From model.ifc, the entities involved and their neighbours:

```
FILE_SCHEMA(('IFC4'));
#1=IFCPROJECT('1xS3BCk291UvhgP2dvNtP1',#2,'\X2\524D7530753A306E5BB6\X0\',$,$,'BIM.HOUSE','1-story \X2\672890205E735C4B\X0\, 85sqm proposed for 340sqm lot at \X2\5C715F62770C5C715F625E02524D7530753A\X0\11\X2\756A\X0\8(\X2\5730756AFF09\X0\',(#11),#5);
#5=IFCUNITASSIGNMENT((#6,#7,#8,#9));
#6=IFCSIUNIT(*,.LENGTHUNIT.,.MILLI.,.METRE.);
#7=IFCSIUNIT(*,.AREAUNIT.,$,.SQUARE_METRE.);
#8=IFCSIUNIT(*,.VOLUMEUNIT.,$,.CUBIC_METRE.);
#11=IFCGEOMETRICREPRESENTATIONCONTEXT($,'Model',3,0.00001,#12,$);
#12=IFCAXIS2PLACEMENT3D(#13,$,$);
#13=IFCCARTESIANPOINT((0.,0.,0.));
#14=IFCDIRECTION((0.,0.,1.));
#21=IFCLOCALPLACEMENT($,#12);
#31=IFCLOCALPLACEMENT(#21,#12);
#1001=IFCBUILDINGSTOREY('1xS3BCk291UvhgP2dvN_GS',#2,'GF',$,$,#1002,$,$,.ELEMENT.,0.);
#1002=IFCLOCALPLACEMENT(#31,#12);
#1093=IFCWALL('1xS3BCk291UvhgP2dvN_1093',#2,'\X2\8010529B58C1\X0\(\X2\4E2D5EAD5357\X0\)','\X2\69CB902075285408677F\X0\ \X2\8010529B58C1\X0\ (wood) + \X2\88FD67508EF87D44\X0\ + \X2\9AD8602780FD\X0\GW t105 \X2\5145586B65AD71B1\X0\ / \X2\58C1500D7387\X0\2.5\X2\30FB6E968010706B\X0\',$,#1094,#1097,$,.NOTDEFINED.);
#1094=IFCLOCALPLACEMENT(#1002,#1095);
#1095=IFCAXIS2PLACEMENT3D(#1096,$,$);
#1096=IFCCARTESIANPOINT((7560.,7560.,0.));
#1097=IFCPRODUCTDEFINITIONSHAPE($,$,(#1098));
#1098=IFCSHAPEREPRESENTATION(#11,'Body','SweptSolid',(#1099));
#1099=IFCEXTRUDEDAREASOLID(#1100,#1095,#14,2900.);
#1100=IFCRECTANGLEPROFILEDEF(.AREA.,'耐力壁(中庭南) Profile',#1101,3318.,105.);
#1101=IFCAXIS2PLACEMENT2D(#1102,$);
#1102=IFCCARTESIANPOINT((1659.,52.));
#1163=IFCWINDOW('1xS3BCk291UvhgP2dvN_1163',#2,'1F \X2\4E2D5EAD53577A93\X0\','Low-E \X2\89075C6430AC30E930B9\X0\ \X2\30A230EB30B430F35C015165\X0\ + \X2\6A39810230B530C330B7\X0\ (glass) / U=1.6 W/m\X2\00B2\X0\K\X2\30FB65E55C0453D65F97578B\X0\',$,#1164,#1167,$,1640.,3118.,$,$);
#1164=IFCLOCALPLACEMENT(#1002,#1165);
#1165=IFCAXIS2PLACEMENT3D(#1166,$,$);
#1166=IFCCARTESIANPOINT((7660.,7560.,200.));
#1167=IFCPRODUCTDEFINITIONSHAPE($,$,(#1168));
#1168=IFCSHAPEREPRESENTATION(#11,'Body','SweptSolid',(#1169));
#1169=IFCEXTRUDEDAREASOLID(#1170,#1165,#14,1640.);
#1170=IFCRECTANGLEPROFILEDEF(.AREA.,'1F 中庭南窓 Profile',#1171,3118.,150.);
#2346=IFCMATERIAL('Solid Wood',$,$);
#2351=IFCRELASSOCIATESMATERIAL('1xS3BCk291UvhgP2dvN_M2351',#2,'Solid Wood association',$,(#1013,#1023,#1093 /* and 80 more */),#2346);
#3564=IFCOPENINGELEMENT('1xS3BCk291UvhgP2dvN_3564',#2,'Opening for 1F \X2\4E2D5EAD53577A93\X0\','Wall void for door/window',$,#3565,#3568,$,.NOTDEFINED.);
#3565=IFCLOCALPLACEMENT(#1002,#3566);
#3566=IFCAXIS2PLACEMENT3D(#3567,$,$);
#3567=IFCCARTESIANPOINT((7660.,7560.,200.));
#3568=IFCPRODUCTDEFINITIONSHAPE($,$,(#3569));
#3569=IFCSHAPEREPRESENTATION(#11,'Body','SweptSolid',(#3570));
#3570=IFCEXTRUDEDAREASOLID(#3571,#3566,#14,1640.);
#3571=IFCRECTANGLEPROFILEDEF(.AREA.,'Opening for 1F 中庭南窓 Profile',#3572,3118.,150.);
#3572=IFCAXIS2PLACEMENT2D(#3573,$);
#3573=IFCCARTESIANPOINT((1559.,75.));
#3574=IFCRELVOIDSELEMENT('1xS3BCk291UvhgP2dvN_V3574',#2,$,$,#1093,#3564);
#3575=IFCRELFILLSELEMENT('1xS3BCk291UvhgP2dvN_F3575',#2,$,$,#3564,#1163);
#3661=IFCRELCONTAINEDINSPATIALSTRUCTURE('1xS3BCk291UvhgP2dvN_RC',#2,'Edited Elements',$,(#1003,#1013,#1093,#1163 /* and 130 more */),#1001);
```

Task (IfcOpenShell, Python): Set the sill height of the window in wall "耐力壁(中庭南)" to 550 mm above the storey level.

```python
import numpy as np
import ifcopenshell
import ifcopenshell.api.geometry
import ifcopenshell.geom
import ifcopenshell.util.element
import ifcopenshell.util.placement
import ifcopenshell.util.shape
import ifcopenshell.util.unit

model = ifcopenshell.open("model.ifc")
unit_scale = ifcopenshell.util.unit.calculate_unit_scale(model)

window = model.by_guid("1xS3BCk291UvhgP2dvN_1163")
opening = window.FillsVoids[0].RelatingOpeningElement
storey = ifcopenshell.util.element.get_container(window, ifc_class="IfcBuildingStorey")
level = ifcopenshell.util.placement.get_local_placement(storey.ObjectPlacement)[2, 3]

# The opening's origin need not be at the sill, so measure its lowest point.
shape = ifcopenshell.geom.create_shape(ifcopenshell.geom.settings(), opening)
bottom = ifcopenshell.util.shape.get_shape_bottom_elevation(shape, shape.geometry) / unit_scale
dz = level + 0.55 / unit_scale - bottom

shift = np.array([0.0, 0.0, dz])
# The window is not placed relative to its opening, so move both.
for product in (opening, window):
    matrix = ifcopenshell.util.placement.get_local_placement(product.ObjectPlacement)
    matrix[:3, 3] += shift
    ifcopenshell.api.geometry.edit_object_placement(model, product=product, matrix=matrix, is_si=False)

print(f"moved by {dz * unit_scale:+.3f} m")

model.write("model_rev.ifc")
```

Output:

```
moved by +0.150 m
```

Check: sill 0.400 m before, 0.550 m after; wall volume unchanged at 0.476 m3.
